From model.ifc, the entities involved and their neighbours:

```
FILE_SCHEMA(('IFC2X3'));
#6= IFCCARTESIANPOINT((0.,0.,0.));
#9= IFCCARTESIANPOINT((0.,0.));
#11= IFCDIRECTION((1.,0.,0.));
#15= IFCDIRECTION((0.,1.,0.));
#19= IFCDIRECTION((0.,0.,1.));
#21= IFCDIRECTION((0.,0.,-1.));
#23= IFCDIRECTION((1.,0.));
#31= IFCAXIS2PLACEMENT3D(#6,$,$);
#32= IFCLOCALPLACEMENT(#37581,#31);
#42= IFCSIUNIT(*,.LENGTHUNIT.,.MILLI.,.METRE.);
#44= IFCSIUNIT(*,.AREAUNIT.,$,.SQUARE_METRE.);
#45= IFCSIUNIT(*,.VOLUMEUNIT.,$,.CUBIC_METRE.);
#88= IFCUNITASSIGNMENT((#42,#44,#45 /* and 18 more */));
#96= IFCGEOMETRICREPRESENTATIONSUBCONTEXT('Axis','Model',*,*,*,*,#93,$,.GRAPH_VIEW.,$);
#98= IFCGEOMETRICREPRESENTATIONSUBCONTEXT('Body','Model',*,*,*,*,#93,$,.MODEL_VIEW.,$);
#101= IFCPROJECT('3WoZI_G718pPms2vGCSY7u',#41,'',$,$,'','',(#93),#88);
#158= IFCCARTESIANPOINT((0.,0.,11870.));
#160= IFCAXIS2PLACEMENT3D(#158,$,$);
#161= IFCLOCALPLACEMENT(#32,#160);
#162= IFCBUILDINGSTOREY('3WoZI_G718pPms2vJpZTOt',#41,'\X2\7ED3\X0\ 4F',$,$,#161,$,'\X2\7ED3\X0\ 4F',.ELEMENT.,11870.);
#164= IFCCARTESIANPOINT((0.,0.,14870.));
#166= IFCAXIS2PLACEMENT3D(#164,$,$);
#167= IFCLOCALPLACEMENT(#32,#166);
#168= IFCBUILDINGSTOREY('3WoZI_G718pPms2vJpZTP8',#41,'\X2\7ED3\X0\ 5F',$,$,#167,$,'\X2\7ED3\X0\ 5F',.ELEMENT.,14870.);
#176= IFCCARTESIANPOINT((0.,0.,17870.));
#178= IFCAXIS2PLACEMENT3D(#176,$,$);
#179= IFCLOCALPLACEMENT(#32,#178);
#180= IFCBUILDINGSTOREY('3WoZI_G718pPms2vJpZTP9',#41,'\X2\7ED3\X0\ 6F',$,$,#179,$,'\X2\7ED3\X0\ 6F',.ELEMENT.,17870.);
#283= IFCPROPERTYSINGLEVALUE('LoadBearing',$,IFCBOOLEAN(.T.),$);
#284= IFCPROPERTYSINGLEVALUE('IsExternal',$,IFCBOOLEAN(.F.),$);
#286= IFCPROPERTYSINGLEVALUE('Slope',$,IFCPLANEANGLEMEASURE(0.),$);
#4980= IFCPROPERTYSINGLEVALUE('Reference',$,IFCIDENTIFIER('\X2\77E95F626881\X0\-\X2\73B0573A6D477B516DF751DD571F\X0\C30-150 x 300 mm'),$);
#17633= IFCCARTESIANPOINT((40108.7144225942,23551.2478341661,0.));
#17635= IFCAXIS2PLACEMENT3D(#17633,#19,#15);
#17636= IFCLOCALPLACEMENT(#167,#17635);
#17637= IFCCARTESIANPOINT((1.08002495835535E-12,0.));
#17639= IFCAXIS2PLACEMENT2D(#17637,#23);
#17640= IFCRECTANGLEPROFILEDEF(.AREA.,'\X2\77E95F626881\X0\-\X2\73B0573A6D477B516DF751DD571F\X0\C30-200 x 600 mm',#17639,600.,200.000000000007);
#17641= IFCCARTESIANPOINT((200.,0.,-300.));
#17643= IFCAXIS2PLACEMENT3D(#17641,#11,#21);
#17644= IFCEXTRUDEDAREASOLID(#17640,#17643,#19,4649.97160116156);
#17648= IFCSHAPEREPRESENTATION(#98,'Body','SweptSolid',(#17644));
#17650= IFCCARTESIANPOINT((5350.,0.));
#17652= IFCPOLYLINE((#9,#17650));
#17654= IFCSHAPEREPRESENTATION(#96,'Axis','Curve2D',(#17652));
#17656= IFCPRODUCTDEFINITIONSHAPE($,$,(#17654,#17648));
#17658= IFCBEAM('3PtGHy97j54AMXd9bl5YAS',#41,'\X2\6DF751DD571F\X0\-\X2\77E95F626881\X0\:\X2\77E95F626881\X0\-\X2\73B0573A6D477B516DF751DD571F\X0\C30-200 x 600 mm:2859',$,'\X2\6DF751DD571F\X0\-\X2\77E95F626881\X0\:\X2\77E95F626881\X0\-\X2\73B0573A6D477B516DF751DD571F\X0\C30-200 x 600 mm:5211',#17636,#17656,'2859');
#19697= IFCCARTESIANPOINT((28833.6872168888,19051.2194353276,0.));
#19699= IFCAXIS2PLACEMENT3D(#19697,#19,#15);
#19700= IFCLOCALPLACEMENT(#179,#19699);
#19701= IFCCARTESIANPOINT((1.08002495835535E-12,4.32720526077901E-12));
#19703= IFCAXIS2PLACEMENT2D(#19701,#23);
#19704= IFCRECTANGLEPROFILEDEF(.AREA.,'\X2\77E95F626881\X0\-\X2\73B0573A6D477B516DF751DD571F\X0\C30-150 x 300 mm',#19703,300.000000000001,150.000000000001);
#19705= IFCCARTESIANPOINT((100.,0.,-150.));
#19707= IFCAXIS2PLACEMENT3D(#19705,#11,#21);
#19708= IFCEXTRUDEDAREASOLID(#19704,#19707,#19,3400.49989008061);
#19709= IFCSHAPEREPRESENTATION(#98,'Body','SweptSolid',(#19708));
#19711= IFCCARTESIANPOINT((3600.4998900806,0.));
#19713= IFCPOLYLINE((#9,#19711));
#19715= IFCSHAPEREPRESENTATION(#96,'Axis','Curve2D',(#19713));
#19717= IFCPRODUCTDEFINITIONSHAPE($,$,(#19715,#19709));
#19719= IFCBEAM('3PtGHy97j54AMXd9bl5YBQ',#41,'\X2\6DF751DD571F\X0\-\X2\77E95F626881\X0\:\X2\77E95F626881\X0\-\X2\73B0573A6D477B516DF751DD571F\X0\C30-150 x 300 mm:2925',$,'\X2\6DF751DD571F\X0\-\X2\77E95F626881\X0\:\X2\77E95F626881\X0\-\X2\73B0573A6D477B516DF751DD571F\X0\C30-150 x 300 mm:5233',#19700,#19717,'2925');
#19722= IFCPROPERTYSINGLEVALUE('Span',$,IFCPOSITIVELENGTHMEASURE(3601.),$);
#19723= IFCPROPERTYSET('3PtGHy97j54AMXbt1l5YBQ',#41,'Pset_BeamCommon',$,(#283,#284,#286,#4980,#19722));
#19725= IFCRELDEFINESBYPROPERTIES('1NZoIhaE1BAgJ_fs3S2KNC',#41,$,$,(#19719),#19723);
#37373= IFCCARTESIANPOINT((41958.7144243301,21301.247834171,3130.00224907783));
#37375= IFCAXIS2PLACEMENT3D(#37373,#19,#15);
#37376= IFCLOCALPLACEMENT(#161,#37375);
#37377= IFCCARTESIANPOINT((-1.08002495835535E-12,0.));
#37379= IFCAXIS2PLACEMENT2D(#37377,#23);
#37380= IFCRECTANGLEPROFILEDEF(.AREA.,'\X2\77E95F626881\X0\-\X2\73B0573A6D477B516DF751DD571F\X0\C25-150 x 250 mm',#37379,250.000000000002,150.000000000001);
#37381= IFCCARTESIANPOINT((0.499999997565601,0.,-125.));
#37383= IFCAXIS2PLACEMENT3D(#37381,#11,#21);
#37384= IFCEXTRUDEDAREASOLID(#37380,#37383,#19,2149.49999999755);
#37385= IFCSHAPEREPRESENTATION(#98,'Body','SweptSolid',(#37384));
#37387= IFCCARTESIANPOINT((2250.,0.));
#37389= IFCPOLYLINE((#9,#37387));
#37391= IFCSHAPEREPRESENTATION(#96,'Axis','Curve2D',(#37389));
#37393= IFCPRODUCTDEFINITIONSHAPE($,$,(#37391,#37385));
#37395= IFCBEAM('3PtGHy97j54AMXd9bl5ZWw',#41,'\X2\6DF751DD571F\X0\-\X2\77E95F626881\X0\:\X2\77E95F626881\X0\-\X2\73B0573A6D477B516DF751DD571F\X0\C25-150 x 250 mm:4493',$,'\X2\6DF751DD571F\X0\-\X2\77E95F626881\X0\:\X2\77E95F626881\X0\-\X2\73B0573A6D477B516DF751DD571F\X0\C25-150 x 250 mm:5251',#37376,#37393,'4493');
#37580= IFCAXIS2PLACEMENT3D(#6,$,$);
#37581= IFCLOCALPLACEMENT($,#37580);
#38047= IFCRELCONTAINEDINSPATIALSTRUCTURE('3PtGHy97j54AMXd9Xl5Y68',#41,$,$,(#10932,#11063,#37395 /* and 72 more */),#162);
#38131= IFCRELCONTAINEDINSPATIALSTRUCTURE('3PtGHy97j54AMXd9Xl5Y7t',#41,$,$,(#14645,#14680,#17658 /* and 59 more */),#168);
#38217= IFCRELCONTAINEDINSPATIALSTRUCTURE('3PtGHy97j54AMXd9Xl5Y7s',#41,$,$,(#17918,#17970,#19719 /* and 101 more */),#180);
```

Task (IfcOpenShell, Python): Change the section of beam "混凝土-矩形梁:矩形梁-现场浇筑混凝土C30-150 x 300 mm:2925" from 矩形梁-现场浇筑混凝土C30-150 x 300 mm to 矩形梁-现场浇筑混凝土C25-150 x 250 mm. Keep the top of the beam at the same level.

```python
import ifcopenshell
import ifcopenshell.api.pset
import ifcopenshell.util.element
import ifcopenshell.util.representation

model = ifcopenshell.open("model.ifc")

member = model.by_guid("3PtGHy97j54AMXd9bl5YBQ")
source = next(p for p in model.by_type("IfcRectangleProfileDef") if p.ProfileName == "矩形梁-现场浇筑混凝土C25-150 x 250 mm")

body = ifcopenshell.util.representation.get_representation(member, "Model", "Body")
solid = body.Items[0]
old_profile = solid.SweptArea

# Copy the section's sizes but keep this member's own profile position.
profile = ifcopenshell.util.element.copy(model, source)
# Profiles are centred, so shift by half the change in depth to hold the top.
shift = (old_profile.XDim - profile.XDim) / 2
x, y = old_profile.Position.Location.Coordinates
up = (-1.0, 0.0)  # upwards, in the solid's own plane
location = model.createIfcCartesianPoint((x + up[0] * shift, y + up[1] * shift))
profile.Position = model.createIfcAxis2Placement2D(location, old_profile.Position.RefDirection)
solid.SweptArea = profile
if not model.get_total_inverses(old_profile):
    ifcopenshell.util.element.remove_deep2(model, old_profile)
member.Name = member.Name.replace("矩形梁-现场浇筑混凝土C30-150 x 300 mm", "矩形梁-现场浇筑混凝土C25-150 x 250 mm")
member.ObjectType = member.ObjectType.replace("矩形梁-现场浇筑混凝土C30-150 x 300 mm", "矩形梁-现场浇筑混凝土C25-150 x 250 mm")
pset = model.by_id(ifcopenshell.util.element.get_pset(member, "Pset_BeamCommon", should_inherit=False)["id"])
ifcopenshell.api.pset.edit_pset(model, pset=pset, properties={"Reference": "矩形梁-现场浇筑混凝土C25-150 x 250 mm"})

print(solid.SweptArea)

model.write("model_edited.ifc")
```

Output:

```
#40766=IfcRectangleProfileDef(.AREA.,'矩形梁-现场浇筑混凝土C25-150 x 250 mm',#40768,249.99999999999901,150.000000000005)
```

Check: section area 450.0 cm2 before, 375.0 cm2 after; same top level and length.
